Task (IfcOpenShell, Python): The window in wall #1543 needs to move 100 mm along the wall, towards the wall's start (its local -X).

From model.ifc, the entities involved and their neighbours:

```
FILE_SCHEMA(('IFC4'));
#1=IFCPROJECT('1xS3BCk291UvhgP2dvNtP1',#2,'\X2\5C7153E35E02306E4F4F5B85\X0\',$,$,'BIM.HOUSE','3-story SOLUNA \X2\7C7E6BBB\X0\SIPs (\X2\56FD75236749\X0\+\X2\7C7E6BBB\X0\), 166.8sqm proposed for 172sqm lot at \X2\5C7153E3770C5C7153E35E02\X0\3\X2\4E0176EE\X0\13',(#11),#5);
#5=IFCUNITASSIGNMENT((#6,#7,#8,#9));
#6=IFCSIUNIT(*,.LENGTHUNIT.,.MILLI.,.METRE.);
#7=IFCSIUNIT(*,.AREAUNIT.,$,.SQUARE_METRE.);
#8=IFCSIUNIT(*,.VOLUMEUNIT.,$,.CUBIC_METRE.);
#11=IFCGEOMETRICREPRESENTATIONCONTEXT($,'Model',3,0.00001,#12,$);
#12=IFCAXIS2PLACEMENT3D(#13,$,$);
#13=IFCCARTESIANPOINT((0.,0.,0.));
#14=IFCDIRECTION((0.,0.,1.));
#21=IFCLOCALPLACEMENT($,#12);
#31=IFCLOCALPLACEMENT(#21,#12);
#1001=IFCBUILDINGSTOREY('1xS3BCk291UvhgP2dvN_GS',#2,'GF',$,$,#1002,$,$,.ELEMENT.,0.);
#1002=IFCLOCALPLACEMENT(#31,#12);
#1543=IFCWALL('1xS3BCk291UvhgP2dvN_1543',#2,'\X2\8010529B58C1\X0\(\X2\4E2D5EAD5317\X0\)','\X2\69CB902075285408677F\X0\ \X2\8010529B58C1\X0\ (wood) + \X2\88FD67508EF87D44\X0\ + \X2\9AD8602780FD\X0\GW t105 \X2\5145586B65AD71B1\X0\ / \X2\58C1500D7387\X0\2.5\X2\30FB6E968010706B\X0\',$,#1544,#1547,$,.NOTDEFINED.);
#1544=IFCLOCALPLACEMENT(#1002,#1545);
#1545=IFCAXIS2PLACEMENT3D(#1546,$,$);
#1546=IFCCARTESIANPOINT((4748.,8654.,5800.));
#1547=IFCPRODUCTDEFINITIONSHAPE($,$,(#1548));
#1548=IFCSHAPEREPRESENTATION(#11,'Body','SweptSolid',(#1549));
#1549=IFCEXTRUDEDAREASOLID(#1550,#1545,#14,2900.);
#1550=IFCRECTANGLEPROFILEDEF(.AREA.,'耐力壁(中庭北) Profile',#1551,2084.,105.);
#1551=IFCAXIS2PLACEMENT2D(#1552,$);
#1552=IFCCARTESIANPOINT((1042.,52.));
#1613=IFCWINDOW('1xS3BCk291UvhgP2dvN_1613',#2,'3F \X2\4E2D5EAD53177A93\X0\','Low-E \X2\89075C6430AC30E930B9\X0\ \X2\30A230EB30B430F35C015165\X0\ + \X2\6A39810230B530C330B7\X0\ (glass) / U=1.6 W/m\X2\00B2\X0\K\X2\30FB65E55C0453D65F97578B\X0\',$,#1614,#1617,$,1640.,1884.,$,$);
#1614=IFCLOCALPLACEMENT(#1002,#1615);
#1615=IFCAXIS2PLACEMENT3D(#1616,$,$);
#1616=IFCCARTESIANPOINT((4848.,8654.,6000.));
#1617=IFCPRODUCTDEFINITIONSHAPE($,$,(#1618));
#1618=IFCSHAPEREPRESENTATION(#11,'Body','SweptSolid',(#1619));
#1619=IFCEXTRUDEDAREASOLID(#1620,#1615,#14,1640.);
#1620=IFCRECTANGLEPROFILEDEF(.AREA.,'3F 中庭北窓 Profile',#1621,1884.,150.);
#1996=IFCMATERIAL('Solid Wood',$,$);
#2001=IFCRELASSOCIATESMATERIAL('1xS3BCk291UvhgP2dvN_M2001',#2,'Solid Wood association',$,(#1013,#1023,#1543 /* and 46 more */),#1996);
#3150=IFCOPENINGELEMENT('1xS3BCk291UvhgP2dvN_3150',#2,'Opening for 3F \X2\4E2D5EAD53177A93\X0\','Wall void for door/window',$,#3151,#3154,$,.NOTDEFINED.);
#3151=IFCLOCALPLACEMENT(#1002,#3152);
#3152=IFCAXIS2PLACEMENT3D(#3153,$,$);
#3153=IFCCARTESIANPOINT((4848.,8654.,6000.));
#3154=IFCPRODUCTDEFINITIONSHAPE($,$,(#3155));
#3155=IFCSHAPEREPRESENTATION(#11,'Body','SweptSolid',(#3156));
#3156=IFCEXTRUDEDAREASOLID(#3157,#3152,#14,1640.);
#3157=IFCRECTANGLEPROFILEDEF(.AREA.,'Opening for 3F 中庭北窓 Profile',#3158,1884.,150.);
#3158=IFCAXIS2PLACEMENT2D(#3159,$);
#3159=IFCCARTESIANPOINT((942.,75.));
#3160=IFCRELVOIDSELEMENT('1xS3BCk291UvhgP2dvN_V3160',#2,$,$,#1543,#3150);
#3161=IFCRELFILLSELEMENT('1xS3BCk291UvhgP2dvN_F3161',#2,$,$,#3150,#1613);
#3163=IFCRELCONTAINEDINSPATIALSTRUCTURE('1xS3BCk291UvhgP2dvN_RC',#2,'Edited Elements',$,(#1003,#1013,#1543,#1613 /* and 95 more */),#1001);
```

```python
import ifcopenshell
import ifcopenshell.api.geometry
import ifcopenshell.util.placement
import ifcopenshell.util.unit

model = ifcopenshell.open("model.ifc")
unit_scale = ifcopenshell.util.unit.calculate_unit_scale(model)

window = model.by_guid("1xS3BCk291UvhgP2dvN_1613")
opening = window.FillsVoids[0].RelatingOpeningElement
wall = opening.VoidsElements[0].RelatingBuildingElement

wall_matrix = ifcopenshell.util.placement.get_local_placement(wall.ObjectPlacement)
shift = wall_matrix[:3, 0] * -0.1 / unit_scale
before = ifcopenshell.util.placement.get_local_placement(window.ObjectPlacement)[:3, 3].copy()

# The window is not placed relative to its opening, so move both.
for product in (opening, window):
    matrix = ifcopenshell.util.placement.get_local_placement(product.ObjectPlacement)
    matrix[:3, 3] += shift
    ifcopenshell.api.geometry.edit_object_placement(model, product=product, matrix=matrix, is_si=False)

after = ifcopenshell.util.placement.get_local_placement(window.ObjectPlacement)[:3, 3]
print("window moved by", (after - before).round(3) + 0.0)

model.write("model_rev.ifc")
```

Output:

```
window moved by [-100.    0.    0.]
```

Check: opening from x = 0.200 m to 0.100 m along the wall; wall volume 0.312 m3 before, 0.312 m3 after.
